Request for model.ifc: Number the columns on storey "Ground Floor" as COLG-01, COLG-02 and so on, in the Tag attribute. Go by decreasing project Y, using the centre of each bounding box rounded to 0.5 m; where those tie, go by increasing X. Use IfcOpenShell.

First a look at what the model holds.

```python
import ifcopenshell
import ifcopenshell.util.element
import ifcopenshell.util.placement

model = ifcopenshell.open("model.ifc")
print(model.schema)
storey = next(s for s in model.by_type("IfcBuildingStorey") if s.Name == "Ground Floor")
columns = [e for e in ifcopenshell.util.element.get_decomposition(storey) if e.is_a("IfcColumn")]
for e in sorted(columns, key=lambda e: e.id()):
    origin = ifcopenshell.util.placement.get_local_placement(e.ObjectPlacement)[:3, 3]
    print(e.id(), e.Tag, e.Name, origin.round(2) + 0.0, sep=" | ")
```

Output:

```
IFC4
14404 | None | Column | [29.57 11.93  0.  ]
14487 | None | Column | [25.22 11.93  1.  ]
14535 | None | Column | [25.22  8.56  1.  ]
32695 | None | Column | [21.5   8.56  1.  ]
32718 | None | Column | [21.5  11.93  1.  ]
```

```python
import ifcopenshell
import ifcopenshell.geom
import ifcopenshell.util.element
import ifcopenshell.util.shape

model = ifcopenshell.open("model.ifc")
settings = ifcopenshell.geom.settings()
settings.set("use-world-coords", True)


def centre(element):
    shape = ifcopenshell.geom.create_shape(settings, element)
    return ifcopenshell.util.shape.get_bbox_centroid(shape.geometry)


storey = next(s for s in model.by_type("IfcBuildingStorey") if s.Name == "Ground Floor")
columns = [e for e in ifcopenshell.util.element.get_decomposition(storey) if e.is_a("IfcColumn")]

# Insertion points can sit at a corner or the storey origin, so sort by the geometry (in metres).
centres = {e: centre(e) for e in columns}
columns.sort(key=lambda e: (-round(centres[e][1] / 0.5), centres[e][0]))

for i, e in enumerate(columns, start=1):
    number = f"COLG-{i:02d}"
    e.Tag = number
    print(e.id(), number)

model.write("model_updated.ifc")
```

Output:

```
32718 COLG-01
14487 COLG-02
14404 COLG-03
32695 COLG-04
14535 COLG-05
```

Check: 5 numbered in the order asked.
